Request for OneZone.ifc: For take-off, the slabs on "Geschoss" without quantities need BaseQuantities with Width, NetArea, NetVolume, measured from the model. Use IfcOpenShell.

First a look at what the model holds.

```python
import ifcopenshell
import ifcopenshell.util.element
import ifcopenshell.util.unit

model = ifcopenshell.open("OneZone.ifc")
print(model.schema)
for unit_type in ("LENGTHUNIT", "AREAUNIT", "VOLUMEUNIT"):
    print(unit_type, ifcopenshell.util.unit.calculate_unit_scale(model, unit_type))
storey = next(s for s in model.by_type("IfcBuildingStorey") if s.Name == "Geschoss")
slabs = [e for e in ifcopenshell.util.element.get_decomposition(storey) if e.is_a("IfcSlab")]
for e in sorted(slabs, key=lambda e: e.id()):
    print(e.id(), e.is_a(), e.Name, list(ifcopenshell.util.element.get_psets(e, qtos_only=True)), sep=" | ")
```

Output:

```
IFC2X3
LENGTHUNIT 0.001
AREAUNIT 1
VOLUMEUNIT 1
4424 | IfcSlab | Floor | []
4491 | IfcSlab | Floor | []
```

```python
import ifcopenshell
import ifcopenshell.api.pset
import ifcopenshell.geom
import ifcopenshell.util.element
import ifcopenshell.util.shape
import ifcopenshell.util.unit

model = ifcopenshell.open("OneZone.ifc")
unit_scale = ifcopenshell.util.unit.calculate_unit_scale(model)
area_scale = ifcopenshell.util.unit.calculate_unit_scale(model, "AREAUNIT")
volume_scale = ifcopenshell.util.unit.calculate_unit_scale(model, "VOLUMEUNIT")
settings = ifcopenshell.geom.settings()

storey = next(s for s in model.by_type("IfcBuildingStorey") if s.Name == "Geschoss")
slabs = [e for e in ifcopenshell.util.element.get_decomposition(storey) if e.is_a("IfcSlab")]

for e in sorted(slabs, key=lambda e: e.id()):
    if ifcopenshell.util.element.get_psets(e, qtos_only=True, should_inherit=False):
        continue
    # Geometry comes back in metres, in the element's own axes.
    shape = ifcopenshell.geom.create_shape(settings, e)
    values = {
        "Width": ifcopenshell.util.shape.get_z(shape.geometry) / unit_scale,
        "NetArea": ifcopenshell.util.shape.get_footprint_area(shape.geometry) / area_scale,
        "NetVolume": ifcopenshell.util.shape.get_volume(shape.geometry) / volume_scale,
    }
    qto = ifcopenshell.api.pset.add_qto(model, product=e, name="BaseQuantities")
    ifcopenshell.api.pset.edit_qto(model, qto=qto, properties=values)
    print(e.id(), {k: round(v, 3) for k, v in values.items()})

model.write("OneZone_updated.ifc")
```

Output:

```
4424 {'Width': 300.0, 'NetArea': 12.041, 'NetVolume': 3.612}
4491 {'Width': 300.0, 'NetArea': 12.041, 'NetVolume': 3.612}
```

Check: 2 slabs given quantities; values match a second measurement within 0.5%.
